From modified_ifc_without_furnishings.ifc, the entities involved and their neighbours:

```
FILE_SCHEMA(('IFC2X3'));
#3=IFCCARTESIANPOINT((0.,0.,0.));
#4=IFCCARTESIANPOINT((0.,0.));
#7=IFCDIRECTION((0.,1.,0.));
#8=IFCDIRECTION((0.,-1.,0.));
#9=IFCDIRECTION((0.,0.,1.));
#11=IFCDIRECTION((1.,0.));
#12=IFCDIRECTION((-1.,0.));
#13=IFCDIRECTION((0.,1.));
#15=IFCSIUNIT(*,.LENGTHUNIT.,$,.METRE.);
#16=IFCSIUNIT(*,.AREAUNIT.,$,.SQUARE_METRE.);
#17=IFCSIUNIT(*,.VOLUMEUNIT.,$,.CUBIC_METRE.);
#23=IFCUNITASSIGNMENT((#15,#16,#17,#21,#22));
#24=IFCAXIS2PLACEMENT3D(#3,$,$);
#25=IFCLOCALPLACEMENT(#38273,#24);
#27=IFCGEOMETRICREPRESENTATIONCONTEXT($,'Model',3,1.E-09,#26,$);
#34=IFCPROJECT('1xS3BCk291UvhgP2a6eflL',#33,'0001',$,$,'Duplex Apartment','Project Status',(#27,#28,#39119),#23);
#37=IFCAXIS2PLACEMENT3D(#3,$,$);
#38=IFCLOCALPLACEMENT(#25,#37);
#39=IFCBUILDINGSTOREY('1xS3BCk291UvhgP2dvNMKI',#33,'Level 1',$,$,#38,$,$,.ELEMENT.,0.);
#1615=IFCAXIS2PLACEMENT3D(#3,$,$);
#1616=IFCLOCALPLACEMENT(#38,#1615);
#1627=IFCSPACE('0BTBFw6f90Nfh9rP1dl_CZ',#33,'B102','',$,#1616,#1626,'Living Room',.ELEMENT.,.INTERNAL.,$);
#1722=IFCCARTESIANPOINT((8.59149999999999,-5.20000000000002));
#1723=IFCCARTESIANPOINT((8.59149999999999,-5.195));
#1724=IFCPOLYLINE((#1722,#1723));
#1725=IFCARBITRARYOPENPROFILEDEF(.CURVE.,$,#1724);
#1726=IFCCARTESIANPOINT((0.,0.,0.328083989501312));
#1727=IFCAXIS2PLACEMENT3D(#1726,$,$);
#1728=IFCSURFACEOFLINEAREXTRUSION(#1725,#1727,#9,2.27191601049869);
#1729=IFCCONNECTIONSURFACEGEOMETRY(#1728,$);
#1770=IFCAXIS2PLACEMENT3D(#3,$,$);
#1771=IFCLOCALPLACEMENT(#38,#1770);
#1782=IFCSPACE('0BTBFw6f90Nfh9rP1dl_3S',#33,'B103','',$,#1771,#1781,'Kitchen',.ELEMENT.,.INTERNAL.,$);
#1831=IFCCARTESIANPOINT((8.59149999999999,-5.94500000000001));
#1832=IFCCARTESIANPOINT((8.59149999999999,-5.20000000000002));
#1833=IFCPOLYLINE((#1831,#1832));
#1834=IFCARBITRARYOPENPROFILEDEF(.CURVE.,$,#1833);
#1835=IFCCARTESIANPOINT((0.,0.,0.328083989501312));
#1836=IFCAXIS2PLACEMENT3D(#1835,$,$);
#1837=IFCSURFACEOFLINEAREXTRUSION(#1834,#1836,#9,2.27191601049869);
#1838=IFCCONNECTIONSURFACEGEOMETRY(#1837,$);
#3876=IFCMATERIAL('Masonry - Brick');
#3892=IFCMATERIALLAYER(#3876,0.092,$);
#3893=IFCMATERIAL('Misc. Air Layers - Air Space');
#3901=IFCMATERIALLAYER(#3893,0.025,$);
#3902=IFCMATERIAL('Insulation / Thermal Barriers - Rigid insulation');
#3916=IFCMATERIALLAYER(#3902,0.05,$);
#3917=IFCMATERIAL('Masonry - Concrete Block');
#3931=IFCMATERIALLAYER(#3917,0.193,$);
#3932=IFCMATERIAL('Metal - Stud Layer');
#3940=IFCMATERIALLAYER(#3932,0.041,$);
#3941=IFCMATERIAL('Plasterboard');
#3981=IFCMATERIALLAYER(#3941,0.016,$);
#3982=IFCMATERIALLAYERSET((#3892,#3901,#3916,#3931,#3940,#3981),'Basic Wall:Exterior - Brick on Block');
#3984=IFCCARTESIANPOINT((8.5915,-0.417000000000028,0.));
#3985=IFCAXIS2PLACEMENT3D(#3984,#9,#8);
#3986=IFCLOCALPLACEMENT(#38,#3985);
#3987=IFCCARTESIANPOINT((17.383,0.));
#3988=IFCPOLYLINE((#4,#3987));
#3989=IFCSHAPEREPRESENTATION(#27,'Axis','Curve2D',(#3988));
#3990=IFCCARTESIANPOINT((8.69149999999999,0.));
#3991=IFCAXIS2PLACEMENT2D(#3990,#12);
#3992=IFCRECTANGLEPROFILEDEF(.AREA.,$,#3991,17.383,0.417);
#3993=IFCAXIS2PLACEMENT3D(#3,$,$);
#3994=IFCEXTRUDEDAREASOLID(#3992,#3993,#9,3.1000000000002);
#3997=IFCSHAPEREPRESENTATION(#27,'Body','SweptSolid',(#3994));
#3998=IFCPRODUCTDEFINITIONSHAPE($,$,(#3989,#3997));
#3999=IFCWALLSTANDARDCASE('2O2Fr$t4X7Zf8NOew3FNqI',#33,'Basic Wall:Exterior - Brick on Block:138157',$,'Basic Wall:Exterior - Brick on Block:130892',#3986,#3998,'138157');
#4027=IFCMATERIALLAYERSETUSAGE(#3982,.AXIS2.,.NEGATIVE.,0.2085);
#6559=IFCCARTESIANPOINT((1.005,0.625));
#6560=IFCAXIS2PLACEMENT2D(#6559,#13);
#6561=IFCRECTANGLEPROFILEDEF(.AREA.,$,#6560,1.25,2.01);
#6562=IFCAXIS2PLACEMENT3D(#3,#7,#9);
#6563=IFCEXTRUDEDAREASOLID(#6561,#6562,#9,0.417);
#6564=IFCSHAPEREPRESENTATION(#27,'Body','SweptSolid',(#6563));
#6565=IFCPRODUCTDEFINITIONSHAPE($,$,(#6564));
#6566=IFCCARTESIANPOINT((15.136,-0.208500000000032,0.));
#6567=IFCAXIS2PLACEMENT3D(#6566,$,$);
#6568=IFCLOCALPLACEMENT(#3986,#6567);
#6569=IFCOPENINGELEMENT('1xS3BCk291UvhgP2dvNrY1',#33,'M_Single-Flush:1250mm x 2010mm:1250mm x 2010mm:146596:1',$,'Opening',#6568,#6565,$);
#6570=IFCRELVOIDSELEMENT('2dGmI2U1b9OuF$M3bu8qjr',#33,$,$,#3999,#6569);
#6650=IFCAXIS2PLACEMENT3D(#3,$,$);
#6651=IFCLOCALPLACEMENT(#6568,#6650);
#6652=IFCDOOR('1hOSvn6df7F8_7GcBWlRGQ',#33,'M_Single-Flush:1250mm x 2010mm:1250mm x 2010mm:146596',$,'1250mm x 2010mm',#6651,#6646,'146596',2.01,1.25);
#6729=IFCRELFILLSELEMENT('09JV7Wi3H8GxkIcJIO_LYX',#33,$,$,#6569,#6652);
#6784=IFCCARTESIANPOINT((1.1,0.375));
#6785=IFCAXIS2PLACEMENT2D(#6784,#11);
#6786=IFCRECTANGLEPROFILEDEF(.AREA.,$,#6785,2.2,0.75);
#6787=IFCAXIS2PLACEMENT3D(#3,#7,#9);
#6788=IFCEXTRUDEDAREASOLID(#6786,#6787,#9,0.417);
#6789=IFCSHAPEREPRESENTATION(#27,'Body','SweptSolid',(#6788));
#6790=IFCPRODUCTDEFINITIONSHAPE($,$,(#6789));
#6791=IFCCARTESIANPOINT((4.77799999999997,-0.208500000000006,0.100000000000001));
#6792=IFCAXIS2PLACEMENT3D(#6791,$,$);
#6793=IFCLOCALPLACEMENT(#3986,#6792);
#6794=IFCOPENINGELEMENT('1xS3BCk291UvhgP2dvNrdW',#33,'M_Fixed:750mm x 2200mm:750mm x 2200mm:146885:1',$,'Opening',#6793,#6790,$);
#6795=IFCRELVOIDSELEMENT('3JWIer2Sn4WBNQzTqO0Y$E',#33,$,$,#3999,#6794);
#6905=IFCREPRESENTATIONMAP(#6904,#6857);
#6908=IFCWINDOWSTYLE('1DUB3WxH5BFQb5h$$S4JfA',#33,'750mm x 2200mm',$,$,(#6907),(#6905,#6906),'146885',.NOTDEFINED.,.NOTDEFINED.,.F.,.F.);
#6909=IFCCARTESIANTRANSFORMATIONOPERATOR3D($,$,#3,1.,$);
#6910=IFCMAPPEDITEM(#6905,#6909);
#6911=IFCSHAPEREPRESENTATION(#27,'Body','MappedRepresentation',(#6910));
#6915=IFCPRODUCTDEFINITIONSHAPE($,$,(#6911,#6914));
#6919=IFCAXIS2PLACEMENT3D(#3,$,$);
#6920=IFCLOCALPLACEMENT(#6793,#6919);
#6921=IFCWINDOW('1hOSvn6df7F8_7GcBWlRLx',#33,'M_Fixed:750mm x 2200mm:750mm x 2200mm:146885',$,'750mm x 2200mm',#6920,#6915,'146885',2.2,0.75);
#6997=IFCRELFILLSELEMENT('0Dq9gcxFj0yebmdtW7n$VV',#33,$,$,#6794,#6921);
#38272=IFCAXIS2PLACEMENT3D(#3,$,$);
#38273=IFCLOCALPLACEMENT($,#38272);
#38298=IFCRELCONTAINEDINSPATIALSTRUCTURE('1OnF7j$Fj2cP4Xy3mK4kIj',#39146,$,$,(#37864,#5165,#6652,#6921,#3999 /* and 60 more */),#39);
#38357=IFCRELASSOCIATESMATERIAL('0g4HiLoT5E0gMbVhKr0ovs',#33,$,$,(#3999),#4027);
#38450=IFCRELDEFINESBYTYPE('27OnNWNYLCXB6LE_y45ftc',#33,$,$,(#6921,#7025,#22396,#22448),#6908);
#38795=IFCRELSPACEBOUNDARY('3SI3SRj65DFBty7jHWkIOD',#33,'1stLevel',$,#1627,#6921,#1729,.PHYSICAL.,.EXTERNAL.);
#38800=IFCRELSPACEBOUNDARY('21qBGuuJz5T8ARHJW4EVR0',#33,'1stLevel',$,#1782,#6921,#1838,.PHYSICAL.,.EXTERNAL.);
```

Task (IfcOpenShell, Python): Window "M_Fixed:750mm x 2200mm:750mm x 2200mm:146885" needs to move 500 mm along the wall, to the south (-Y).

```python
import numpy as np
import ifcopenshell
import ifcopenshell.api.geometry
import ifcopenshell.util.placement

model = ifcopenshell.open("modified_ifc_without_furnishings.ifc")

window = model.by_guid("1hOSvn6df7F8_7GcBWlRLx")
opening = window.FillsVoids[0].RelatingOpeningElement
wall = opening.VoidsElements[0].RelatingBuildingElement

wall_matrix = ifcopenshell.util.placement.get_local_placement(wall.ObjectPlacement)
shift = wall_matrix[:3, 0] * 0.5
before = ifcopenshell.util.placement.get_local_placement(window.ObjectPlacement)[:3, 3].copy()

# The window is placed relative to its opening, so it follows when the opening moves.
matrix = ifcopenshell.util.placement.get_local_placement(opening.ObjectPlacement)
matrix[:3, 3] += shift
ifcopenshell.api.geometry.edit_object_placement(
    model, product=opening, matrix=matrix, is_si=False, should_transform_children=True
)

# Space boundary surfaces are stored in each space's coordinates; move them too.
for rel in window.ProvidesBoundaries:
    if not rel.ConnectionGeometry:
        continue
    surface = rel.ConnectionGeometry.SurfaceOnRelatingElement
    space_matrix = ifcopenshell.util.placement.get_local_placement(rel.RelatingSpace.ObjectPlacement)
    point = np.array(surface.Position.Location.Coordinates) + space_matrix[:3, :3].T @ shift
    surface.Position = model.createIfcAxis2Placement3D(
        model.createIfcCartesianPoint(point.tolist()), surface.Position.Axis, surface.Position.RefDirection
    )

after = ifcopenshell.util.placement.get_local_placement(window.ObjectPlacement)[:3, 3]
print("window moved by", (after - before).round(3) + 0.0)

model.write("modified_ifc_without_furnishings_rev.ifc")
```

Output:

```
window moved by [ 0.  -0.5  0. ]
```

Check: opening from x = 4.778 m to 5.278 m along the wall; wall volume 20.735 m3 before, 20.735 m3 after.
